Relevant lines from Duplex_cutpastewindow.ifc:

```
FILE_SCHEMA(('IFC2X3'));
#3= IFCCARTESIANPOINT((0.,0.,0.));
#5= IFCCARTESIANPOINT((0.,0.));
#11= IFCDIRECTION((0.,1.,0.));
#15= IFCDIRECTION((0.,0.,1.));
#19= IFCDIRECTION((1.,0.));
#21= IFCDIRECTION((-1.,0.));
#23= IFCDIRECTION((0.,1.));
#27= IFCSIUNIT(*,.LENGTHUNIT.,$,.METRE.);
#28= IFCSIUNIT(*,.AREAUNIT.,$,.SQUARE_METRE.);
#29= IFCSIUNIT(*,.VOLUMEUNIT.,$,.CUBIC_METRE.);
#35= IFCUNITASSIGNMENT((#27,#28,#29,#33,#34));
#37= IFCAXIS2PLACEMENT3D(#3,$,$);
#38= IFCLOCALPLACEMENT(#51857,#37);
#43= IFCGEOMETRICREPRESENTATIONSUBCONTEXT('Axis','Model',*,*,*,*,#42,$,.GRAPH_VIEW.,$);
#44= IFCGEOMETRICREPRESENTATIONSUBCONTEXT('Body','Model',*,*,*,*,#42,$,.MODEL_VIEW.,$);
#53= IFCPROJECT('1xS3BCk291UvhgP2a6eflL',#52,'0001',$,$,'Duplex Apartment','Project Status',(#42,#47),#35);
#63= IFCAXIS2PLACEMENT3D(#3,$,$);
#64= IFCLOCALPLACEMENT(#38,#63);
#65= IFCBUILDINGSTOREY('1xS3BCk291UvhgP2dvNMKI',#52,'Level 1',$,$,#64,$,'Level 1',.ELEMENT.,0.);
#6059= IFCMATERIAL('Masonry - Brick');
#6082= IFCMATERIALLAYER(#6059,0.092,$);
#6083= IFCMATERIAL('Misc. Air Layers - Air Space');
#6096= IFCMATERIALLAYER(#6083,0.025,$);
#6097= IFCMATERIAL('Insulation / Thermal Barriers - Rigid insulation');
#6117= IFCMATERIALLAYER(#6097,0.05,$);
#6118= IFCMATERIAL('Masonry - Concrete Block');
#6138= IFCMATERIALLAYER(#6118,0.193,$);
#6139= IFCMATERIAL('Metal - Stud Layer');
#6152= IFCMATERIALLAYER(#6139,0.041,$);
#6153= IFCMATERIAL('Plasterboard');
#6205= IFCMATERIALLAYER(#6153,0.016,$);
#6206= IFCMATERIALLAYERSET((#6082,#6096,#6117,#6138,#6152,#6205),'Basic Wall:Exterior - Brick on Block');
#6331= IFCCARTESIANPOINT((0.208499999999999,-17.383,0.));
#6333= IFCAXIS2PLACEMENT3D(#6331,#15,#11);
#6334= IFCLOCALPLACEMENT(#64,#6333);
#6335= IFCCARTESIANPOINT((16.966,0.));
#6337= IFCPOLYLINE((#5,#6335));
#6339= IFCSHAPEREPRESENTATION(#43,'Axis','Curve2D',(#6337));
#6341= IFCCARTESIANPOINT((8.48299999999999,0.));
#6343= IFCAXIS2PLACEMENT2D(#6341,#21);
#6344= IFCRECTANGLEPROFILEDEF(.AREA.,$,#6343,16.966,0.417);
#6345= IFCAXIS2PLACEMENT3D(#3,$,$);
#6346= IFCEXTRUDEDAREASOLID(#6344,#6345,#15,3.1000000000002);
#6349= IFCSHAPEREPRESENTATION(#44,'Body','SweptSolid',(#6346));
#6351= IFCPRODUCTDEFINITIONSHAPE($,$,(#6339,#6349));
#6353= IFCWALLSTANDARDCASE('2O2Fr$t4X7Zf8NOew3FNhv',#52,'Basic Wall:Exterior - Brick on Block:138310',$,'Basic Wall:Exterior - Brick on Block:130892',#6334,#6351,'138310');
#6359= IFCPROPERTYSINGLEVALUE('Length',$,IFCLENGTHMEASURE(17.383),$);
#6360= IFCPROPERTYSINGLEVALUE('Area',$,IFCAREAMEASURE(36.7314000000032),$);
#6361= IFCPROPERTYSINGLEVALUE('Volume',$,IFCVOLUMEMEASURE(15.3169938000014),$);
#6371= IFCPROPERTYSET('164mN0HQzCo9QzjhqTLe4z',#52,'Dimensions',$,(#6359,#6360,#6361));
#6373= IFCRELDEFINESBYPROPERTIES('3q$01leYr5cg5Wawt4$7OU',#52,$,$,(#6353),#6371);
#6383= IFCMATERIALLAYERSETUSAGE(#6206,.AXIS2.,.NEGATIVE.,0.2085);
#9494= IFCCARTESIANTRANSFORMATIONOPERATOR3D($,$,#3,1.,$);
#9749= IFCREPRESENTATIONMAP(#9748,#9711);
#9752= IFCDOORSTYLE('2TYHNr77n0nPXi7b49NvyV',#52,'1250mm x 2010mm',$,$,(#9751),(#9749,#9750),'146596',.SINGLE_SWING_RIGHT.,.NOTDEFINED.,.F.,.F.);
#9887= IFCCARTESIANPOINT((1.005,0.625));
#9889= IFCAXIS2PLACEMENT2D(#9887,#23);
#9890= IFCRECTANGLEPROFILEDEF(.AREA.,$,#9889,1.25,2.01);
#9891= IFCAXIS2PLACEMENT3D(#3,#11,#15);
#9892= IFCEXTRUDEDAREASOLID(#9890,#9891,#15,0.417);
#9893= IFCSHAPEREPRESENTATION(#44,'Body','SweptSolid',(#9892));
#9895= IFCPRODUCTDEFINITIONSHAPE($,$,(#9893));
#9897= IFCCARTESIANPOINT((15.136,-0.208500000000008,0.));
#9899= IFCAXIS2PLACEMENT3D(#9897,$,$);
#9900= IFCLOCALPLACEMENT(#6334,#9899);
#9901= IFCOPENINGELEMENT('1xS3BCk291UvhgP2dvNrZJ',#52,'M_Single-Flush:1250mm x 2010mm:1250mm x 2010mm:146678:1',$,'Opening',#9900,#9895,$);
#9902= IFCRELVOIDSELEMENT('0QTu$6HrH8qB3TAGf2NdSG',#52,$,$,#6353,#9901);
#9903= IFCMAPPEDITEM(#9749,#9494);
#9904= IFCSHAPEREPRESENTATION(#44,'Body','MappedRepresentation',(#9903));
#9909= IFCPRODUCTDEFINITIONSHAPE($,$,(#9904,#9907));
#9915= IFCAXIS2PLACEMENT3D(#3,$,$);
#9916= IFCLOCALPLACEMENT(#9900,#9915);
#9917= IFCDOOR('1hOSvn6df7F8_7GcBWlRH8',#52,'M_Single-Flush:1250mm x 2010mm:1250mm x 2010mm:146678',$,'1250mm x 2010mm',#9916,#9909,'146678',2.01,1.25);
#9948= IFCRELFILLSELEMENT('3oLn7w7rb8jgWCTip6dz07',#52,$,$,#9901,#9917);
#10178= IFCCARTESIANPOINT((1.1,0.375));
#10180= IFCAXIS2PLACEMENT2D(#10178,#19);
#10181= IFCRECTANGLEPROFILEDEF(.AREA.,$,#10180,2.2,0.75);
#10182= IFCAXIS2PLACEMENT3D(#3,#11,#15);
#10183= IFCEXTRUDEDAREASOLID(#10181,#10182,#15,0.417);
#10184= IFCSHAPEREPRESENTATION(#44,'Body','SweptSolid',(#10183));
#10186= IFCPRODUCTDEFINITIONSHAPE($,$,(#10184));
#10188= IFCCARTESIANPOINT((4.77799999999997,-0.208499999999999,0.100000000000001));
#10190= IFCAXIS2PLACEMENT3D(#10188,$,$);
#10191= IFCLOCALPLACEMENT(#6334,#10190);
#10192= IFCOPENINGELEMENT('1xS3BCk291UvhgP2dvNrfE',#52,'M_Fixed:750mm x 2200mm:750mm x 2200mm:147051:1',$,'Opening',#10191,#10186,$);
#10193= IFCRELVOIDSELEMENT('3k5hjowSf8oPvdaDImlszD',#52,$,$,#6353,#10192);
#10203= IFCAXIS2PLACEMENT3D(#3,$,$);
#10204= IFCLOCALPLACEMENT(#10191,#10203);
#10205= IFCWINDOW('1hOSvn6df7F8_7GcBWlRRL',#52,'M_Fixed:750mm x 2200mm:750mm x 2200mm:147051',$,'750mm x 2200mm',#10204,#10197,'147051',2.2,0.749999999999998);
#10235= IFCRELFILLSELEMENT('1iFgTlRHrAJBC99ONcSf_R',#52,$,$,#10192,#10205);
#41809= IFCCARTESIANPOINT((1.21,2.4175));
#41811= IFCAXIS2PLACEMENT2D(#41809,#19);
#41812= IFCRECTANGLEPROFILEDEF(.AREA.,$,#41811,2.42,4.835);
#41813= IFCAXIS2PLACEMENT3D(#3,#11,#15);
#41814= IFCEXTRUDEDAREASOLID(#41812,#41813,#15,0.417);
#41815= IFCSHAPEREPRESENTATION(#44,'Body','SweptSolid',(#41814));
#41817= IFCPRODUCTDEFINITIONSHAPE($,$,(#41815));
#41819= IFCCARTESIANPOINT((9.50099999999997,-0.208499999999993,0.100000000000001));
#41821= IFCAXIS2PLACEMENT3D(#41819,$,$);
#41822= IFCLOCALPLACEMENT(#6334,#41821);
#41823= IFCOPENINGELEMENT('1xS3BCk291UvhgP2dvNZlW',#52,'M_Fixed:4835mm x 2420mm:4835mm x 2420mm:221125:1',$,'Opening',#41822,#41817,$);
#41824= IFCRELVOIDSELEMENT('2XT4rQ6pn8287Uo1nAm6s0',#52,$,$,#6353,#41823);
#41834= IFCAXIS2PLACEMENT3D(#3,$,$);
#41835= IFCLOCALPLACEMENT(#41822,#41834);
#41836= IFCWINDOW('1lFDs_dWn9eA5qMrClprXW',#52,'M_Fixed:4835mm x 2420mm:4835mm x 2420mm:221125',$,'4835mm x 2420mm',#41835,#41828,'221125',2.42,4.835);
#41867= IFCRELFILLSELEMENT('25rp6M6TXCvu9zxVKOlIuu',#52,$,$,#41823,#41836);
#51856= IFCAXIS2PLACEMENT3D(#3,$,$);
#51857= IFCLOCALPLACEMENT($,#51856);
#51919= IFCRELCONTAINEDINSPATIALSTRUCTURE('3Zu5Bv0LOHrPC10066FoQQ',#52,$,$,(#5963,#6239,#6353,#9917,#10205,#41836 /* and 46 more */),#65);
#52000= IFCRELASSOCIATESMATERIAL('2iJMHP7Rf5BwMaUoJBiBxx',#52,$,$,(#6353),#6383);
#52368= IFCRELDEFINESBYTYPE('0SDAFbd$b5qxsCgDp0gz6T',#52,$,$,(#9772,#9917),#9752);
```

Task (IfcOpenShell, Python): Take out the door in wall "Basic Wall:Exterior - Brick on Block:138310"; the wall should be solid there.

```python
import ifcopenshell
import ifcopenshell.api.feature
import ifcopenshell.api.pset
import ifcopenshell.api.root
import ifcopenshell.geom
import ifcopenshell.util.element
import ifcopenshell.util.shape
import ifcopenshell.util.unit

model = ifcopenshell.open("Duplex_cutpastewindow.ifc")
area_scale = ifcopenshell.util.unit.calculate_unit_scale(model, "AREAUNIT")
volume_scale = ifcopenshell.util.unit.calculate_unit_scale(model, "VOLUMEUNIT")
settings = ifcopenshell.geom.settings()


def volume(element):
    """Net volume in cubic metres, openings subtracted."""
    shape = ifcopenshell.geom.create_shape(settings, element)
    return ifcopenshell.util.shape.get_volume(shape.geometry)


door = model.by_guid("1hOSvn6df7F8_7GcBWlRH8")
opening = door.FillsVoids[0].RelatingOpeningElement
wall = opening.VoidsElements[0].RelatingBuildingElement
before = volume(wall)

ifcopenshell.api.root.remove_product(model, product=door)
ifcopenshell.api.feature.remove_feature(model, feature=opening)

after = volume(wall)
thickness = 0.417  # wall thickness in metres

# Update the wall's stored quantities.
pset = model.by_id(ifcopenshell.util.element.get_pset(wall, "Dimensions", should_inherit=False)["id"])
ifcopenshell.api.pset.edit_pset(model, pset=pset, properties={
    "Area": model.create_entity("IfcAreaMeasure", after / thickness / area_scale),
    "Volume": model.create_entity("IfcVolumeMeasure", after / volume_scale),
})

print(f"wall volume {before:.3f} -> {after:.3f} m3")

model.write("Duplex_cutpastewindow_updated.ifc")
```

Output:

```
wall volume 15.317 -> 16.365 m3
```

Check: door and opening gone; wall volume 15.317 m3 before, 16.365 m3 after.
